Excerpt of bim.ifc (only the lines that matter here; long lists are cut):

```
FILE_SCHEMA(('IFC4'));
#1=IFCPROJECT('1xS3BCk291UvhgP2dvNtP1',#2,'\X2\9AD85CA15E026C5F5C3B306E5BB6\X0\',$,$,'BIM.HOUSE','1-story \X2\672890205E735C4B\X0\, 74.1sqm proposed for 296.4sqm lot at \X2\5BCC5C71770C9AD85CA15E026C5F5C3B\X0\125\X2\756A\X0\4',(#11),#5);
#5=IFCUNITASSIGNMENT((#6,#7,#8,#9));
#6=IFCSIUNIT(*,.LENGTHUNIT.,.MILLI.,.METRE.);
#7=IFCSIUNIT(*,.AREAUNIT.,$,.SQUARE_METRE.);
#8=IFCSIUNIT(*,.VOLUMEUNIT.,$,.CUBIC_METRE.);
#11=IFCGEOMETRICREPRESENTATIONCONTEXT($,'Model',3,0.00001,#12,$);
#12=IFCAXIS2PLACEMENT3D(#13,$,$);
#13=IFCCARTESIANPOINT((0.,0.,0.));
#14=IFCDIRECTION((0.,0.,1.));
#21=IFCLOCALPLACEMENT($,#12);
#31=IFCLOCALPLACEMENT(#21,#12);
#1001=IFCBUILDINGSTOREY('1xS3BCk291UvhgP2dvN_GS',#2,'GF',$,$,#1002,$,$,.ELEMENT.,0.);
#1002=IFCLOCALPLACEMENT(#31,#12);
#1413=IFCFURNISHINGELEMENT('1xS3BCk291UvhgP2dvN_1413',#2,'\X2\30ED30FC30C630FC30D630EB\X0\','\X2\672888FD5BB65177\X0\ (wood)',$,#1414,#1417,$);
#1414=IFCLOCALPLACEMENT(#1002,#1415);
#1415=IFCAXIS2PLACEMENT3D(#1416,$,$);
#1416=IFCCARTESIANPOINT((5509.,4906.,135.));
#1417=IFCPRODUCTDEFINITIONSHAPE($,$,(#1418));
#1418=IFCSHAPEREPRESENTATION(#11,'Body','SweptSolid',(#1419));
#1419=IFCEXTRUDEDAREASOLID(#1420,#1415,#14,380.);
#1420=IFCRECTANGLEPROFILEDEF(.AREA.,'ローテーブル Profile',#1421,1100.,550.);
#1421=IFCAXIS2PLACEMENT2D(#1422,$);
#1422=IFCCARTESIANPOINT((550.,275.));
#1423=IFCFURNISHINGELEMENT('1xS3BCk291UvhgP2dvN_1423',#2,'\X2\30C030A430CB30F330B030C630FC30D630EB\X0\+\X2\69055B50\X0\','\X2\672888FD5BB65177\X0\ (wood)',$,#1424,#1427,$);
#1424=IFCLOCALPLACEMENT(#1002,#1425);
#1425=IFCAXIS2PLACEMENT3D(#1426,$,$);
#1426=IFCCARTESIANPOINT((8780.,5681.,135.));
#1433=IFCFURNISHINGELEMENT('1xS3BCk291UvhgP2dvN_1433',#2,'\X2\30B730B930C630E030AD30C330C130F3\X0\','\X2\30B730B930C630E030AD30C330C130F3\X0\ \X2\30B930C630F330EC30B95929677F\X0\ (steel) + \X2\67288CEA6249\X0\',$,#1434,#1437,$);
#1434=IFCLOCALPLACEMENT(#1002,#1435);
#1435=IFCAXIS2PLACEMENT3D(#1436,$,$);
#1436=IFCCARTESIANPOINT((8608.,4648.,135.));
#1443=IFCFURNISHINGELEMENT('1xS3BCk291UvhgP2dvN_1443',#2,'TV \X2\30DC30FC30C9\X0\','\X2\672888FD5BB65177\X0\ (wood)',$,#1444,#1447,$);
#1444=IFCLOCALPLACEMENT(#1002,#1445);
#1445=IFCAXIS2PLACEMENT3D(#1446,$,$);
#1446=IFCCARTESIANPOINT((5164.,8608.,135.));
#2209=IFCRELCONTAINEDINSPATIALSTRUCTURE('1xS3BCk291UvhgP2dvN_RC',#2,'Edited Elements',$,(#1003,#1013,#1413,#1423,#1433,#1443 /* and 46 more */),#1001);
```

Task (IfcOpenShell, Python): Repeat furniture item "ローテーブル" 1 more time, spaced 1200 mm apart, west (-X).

```python
import numpy as np
import ifcopenshell
import ifcopenshell.api.geometry
import ifcopenshell.api.root
import ifcopenshell.util.element
import ifcopenshell.util.placement
import ifcopenshell.util.unit

model = ifcopenshell.open("bim.ifc")
unit_scale = ifcopenshell.util.unit.calculate_unit_scale(model)


def reuse_history(source, copy):
    """copy_class also copies each property set's owner history, people and application; keep the originals."""
    for rel in copy.IsDefinedBy:
        if rel.is_a("IfcRelDefinesByProperties") and (history := rel.RelatingPropertyDefinition.OwnerHistory):
            rel.RelatingPropertyDefinition.OwnerHistory = source.OwnerHistory
            ifcopenshell.util.element.remove_deep2(model, history)


source = model.by_guid("1xS3BCk291UvhgP2dvN_1413")
base = ifcopenshell.util.placement.get_local_placement(source.ObjectPlacement)
step = np.array([-1.0, 0.0, 0.0]) * 1.2 / unit_scale

for i in range(1, 2):
    copy = ifcopenshell.api.root.copy_class(model, product=source)
    copy.Representation = ifcopenshell.util.element.copy_deep(
        model, source.Representation, exclude=["IfcGeometricRepresentationContext", "IfcRepresentationMap"]
    )
    reuse_history(source, copy)
    matrix = base.copy()
    matrix[:3, 3] += i * step
    print("added at", matrix[:3, 3].round(3) + 0.0)
    ifcopenshell.api.geometry.edit_object_placement(model, product=copy, matrix=matrix, is_si=False)

model.write("bim_updated.ifc")
```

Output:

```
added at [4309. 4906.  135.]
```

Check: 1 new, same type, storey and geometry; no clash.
